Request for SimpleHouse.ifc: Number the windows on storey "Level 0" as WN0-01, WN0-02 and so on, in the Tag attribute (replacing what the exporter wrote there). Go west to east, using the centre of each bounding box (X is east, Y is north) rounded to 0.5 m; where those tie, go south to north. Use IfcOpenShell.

First a look at what the model holds.

```python
import ifcopenshell
import ifcopenshell.util.element
import ifcopenshell.util.placement

model = ifcopenshell.open("SimpleHouse.ifc")
print(model.schema)
storey = next(s for s in model.by_type("IfcBuildingStorey") if s.Name == "Level 0")
windows = [e for e in ifcopenshell.util.element.get_decomposition(storey) if e.is_a("IfcWindow")]
for e in sorted(windows, key=lambda e: e.id()):
    origin = ifcopenshell.util.placement.get_local_placement(e.ObjectPlacement)[:3, 3]
    print(e.id(), e.Tag, e.Name, origin.round(2) + 0.0, sep=" | ")
```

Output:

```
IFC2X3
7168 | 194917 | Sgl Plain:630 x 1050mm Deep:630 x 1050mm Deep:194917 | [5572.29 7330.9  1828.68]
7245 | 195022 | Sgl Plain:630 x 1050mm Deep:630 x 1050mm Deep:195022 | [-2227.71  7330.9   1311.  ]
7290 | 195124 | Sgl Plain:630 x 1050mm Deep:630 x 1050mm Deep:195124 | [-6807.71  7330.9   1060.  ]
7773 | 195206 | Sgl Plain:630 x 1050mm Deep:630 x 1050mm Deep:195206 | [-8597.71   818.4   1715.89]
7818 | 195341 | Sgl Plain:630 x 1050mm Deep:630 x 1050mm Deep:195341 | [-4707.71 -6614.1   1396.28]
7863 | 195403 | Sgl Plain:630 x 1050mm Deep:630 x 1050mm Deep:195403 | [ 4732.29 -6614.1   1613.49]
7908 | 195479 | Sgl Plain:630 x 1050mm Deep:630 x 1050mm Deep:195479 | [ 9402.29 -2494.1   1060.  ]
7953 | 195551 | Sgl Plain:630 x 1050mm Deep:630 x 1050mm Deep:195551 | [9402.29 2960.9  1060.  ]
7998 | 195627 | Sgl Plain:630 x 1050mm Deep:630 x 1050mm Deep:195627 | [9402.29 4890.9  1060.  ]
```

```python
import ifcopenshell
import ifcopenshell.geom
import ifcopenshell.util.element
import ifcopenshell.util.shape

model = ifcopenshell.open("SimpleHouse.ifc")
settings = ifcopenshell.geom.settings()
settings.set("use-world-coords", True)


def centre(element):
    shape = ifcopenshell.geom.create_shape(settings, element)
    return ifcopenshell.util.shape.get_bbox_centroid(shape.geometry)


storey = next(s for s in model.by_type("IfcBuildingStorey") if s.Name == "Level 0")
windows = [e for e in ifcopenshell.util.element.get_decomposition(storey) if e.is_a("IfcWindow")]

# Insertion points can sit at a corner or the storey origin, so sort by the geometry (in metres).
centres = {e: centre(e) for e in windows}
windows.sort(key=lambda e: (round(centres[e][0] / 0.5), centres[e][1]))

for i, e in enumerate(windows, start=1):
    number = f"WN0-{i:02d}"
    e.Tag = number
    print(e.id(), number)

model.write("SimpleHouse_edited.ifc")
```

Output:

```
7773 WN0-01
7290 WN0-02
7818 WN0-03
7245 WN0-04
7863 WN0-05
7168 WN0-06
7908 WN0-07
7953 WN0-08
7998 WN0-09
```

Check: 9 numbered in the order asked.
